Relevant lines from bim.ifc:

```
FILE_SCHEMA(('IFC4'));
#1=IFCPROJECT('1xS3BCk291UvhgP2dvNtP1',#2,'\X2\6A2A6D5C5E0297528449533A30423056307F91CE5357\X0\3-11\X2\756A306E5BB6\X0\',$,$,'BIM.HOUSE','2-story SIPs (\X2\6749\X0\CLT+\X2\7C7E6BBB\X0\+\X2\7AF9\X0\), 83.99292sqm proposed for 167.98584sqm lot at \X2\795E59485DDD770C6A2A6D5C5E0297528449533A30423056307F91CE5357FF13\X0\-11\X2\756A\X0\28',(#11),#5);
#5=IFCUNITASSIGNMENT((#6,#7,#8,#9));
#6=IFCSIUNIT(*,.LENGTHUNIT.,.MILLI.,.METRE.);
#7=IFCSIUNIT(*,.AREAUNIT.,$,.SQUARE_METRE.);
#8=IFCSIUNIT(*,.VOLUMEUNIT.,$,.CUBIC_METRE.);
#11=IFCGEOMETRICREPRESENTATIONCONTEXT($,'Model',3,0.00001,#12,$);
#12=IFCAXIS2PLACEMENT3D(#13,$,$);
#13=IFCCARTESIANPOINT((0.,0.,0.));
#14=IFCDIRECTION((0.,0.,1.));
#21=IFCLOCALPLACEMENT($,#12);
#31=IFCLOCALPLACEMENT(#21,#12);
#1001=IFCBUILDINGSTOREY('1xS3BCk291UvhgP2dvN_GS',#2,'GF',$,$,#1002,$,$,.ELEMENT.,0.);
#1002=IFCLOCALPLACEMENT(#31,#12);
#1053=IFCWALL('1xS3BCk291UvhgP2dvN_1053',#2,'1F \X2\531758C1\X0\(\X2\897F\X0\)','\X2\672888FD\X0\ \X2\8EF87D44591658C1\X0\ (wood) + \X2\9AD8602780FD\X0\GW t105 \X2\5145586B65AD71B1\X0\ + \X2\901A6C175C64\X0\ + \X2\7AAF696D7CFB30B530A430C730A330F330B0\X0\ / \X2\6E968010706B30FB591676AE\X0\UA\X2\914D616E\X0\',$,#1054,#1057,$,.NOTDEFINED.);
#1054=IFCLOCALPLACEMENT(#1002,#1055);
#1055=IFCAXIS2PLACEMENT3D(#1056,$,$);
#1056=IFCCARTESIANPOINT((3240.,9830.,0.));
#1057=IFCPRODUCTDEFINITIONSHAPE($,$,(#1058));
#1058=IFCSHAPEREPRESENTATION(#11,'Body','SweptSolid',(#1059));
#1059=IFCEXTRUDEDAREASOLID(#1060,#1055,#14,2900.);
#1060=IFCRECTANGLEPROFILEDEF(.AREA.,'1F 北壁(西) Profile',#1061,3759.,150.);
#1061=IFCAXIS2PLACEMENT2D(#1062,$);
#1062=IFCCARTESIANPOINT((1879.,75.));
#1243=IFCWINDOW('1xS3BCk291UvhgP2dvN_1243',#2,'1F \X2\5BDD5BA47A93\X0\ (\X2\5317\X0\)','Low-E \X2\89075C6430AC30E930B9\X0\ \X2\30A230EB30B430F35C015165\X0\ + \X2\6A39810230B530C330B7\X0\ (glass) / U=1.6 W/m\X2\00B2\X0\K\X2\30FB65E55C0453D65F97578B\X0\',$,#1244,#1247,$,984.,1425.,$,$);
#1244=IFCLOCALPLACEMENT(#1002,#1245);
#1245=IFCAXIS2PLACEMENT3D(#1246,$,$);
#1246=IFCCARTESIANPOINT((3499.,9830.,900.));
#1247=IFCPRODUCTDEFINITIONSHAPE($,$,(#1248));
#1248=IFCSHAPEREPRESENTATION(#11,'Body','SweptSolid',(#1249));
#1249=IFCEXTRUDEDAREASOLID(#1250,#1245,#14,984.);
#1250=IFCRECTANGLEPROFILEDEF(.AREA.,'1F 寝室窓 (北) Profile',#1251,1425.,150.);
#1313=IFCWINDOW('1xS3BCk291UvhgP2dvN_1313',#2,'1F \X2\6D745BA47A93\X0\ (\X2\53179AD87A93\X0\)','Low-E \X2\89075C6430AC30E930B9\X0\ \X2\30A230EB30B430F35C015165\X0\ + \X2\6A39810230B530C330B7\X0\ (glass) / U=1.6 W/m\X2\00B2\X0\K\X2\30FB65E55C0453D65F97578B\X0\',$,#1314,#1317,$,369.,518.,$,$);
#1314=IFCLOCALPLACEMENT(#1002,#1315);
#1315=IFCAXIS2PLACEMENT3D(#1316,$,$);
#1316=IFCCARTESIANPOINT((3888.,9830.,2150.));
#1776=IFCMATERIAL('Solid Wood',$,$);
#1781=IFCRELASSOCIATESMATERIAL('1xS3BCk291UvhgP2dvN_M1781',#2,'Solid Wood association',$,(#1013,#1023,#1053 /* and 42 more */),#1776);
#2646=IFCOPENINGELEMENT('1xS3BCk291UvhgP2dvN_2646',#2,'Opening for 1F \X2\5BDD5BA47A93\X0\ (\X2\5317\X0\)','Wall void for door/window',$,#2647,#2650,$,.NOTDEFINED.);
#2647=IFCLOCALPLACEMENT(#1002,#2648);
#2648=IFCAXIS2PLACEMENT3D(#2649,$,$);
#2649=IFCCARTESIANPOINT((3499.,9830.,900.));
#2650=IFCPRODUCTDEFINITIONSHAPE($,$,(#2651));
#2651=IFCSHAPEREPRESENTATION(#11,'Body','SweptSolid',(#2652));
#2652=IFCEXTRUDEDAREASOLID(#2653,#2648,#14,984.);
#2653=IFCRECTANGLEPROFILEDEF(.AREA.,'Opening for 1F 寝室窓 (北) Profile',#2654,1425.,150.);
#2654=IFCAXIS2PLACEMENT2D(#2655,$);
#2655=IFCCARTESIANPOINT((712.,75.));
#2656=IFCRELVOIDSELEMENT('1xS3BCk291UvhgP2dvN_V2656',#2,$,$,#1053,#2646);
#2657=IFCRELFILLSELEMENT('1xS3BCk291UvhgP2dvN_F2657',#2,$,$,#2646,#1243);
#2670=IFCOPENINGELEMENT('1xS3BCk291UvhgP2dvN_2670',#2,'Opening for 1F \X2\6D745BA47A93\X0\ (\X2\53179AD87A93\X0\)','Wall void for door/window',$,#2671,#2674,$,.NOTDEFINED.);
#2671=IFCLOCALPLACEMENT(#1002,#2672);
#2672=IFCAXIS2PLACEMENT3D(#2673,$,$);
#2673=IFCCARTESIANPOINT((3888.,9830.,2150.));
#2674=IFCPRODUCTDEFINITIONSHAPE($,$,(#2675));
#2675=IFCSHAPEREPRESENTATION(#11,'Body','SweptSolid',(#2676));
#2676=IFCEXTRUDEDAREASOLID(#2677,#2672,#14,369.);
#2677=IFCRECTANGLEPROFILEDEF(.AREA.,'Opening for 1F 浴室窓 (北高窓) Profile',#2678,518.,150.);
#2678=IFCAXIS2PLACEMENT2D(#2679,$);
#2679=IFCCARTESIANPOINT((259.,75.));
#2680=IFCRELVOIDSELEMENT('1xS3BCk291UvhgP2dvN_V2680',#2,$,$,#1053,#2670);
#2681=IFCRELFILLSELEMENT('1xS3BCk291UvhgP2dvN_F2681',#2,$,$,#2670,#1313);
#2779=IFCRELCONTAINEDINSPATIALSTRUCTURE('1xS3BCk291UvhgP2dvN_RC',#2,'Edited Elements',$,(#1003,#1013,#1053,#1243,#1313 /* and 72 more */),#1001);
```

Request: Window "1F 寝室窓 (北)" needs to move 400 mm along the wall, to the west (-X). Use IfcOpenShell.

```python
import ifcopenshell
import ifcopenshell.api.geometry
import ifcopenshell.util.placement
import ifcopenshell.util.unit

model = ifcopenshell.open("bim.ifc")
unit_scale = ifcopenshell.util.unit.calculate_unit_scale(model)

window = model.by_guid("1xS3BCk291UvhgP2dvN_1243")
opening = window.FillsVoids[0].RelatingOpeningElement
wall = opening.VoidsElements[0].RelatingBuildingElement

wall_matrix = ifcopenshell.util.placement.get_local_placement(wall.ObjectPlacement)
shift = wall_matrix[:3, 0] * -0.4 / unit_scale
before = ifcopenshell.util.placement.get_local_placement(window.ObjectPlacement)[:3, 3].copy()

# The window is not placed relative to its opening, so move both.
for product in (opening, window):
    matrix = ifcopenshell.util.placement.get_local_placement(product.ObjectPlacement)
    matrix[:3, 3] += shift
    ifcopenshell.api.geometry.edit_object_placement(model, product=product, matrix=matrix, is_si=False)

after = ifcopenshell.util.placement.get_local_placement(window.ObjectPlacement)[:3, 3]
print("window moved by", (after - before).round(3) + 0.0)

model.write("bim-out.ifc")
```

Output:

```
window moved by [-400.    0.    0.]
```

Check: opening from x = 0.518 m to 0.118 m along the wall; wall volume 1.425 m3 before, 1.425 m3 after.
